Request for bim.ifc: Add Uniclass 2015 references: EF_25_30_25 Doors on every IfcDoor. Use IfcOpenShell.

First a look at what the model holds.

```python
import ifcopenshell

model = ifcopenshell.open("bim.ifc")
print(model.schema)
print("classifications:", [c.Name for c in model.by_type("IfcClassification")])
for ifc_class in ("IfcDoor", "IfcRoof", "IfcStair", "IfcWall", "IfcWindow"):
    print(ifc_class, len(model.by_type(ifc_class)))
```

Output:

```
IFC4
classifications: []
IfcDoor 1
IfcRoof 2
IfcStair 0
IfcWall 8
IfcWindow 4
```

```python
import ifcopenshell
import ifcopenshell.api.classification

model = ifcopenshell.open("bim.ifc")

system = ifcopenshell.api.classification.add_classification(model, classification="Uniclass 2015")

codes = {
    "IfcDoor": ("EF_25_30_25", "Doors"),
}
for ifc_class, (code, name) in codes.items():
    products = model.by_type(ifc_class)
    ifcopenshell.api.classification.add_reference(
        model, products=products, classification=system, identification=code, name=name
    )
    print(code, len(products))

model.write("bim_edited.ifc")
```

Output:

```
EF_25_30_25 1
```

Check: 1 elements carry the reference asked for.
